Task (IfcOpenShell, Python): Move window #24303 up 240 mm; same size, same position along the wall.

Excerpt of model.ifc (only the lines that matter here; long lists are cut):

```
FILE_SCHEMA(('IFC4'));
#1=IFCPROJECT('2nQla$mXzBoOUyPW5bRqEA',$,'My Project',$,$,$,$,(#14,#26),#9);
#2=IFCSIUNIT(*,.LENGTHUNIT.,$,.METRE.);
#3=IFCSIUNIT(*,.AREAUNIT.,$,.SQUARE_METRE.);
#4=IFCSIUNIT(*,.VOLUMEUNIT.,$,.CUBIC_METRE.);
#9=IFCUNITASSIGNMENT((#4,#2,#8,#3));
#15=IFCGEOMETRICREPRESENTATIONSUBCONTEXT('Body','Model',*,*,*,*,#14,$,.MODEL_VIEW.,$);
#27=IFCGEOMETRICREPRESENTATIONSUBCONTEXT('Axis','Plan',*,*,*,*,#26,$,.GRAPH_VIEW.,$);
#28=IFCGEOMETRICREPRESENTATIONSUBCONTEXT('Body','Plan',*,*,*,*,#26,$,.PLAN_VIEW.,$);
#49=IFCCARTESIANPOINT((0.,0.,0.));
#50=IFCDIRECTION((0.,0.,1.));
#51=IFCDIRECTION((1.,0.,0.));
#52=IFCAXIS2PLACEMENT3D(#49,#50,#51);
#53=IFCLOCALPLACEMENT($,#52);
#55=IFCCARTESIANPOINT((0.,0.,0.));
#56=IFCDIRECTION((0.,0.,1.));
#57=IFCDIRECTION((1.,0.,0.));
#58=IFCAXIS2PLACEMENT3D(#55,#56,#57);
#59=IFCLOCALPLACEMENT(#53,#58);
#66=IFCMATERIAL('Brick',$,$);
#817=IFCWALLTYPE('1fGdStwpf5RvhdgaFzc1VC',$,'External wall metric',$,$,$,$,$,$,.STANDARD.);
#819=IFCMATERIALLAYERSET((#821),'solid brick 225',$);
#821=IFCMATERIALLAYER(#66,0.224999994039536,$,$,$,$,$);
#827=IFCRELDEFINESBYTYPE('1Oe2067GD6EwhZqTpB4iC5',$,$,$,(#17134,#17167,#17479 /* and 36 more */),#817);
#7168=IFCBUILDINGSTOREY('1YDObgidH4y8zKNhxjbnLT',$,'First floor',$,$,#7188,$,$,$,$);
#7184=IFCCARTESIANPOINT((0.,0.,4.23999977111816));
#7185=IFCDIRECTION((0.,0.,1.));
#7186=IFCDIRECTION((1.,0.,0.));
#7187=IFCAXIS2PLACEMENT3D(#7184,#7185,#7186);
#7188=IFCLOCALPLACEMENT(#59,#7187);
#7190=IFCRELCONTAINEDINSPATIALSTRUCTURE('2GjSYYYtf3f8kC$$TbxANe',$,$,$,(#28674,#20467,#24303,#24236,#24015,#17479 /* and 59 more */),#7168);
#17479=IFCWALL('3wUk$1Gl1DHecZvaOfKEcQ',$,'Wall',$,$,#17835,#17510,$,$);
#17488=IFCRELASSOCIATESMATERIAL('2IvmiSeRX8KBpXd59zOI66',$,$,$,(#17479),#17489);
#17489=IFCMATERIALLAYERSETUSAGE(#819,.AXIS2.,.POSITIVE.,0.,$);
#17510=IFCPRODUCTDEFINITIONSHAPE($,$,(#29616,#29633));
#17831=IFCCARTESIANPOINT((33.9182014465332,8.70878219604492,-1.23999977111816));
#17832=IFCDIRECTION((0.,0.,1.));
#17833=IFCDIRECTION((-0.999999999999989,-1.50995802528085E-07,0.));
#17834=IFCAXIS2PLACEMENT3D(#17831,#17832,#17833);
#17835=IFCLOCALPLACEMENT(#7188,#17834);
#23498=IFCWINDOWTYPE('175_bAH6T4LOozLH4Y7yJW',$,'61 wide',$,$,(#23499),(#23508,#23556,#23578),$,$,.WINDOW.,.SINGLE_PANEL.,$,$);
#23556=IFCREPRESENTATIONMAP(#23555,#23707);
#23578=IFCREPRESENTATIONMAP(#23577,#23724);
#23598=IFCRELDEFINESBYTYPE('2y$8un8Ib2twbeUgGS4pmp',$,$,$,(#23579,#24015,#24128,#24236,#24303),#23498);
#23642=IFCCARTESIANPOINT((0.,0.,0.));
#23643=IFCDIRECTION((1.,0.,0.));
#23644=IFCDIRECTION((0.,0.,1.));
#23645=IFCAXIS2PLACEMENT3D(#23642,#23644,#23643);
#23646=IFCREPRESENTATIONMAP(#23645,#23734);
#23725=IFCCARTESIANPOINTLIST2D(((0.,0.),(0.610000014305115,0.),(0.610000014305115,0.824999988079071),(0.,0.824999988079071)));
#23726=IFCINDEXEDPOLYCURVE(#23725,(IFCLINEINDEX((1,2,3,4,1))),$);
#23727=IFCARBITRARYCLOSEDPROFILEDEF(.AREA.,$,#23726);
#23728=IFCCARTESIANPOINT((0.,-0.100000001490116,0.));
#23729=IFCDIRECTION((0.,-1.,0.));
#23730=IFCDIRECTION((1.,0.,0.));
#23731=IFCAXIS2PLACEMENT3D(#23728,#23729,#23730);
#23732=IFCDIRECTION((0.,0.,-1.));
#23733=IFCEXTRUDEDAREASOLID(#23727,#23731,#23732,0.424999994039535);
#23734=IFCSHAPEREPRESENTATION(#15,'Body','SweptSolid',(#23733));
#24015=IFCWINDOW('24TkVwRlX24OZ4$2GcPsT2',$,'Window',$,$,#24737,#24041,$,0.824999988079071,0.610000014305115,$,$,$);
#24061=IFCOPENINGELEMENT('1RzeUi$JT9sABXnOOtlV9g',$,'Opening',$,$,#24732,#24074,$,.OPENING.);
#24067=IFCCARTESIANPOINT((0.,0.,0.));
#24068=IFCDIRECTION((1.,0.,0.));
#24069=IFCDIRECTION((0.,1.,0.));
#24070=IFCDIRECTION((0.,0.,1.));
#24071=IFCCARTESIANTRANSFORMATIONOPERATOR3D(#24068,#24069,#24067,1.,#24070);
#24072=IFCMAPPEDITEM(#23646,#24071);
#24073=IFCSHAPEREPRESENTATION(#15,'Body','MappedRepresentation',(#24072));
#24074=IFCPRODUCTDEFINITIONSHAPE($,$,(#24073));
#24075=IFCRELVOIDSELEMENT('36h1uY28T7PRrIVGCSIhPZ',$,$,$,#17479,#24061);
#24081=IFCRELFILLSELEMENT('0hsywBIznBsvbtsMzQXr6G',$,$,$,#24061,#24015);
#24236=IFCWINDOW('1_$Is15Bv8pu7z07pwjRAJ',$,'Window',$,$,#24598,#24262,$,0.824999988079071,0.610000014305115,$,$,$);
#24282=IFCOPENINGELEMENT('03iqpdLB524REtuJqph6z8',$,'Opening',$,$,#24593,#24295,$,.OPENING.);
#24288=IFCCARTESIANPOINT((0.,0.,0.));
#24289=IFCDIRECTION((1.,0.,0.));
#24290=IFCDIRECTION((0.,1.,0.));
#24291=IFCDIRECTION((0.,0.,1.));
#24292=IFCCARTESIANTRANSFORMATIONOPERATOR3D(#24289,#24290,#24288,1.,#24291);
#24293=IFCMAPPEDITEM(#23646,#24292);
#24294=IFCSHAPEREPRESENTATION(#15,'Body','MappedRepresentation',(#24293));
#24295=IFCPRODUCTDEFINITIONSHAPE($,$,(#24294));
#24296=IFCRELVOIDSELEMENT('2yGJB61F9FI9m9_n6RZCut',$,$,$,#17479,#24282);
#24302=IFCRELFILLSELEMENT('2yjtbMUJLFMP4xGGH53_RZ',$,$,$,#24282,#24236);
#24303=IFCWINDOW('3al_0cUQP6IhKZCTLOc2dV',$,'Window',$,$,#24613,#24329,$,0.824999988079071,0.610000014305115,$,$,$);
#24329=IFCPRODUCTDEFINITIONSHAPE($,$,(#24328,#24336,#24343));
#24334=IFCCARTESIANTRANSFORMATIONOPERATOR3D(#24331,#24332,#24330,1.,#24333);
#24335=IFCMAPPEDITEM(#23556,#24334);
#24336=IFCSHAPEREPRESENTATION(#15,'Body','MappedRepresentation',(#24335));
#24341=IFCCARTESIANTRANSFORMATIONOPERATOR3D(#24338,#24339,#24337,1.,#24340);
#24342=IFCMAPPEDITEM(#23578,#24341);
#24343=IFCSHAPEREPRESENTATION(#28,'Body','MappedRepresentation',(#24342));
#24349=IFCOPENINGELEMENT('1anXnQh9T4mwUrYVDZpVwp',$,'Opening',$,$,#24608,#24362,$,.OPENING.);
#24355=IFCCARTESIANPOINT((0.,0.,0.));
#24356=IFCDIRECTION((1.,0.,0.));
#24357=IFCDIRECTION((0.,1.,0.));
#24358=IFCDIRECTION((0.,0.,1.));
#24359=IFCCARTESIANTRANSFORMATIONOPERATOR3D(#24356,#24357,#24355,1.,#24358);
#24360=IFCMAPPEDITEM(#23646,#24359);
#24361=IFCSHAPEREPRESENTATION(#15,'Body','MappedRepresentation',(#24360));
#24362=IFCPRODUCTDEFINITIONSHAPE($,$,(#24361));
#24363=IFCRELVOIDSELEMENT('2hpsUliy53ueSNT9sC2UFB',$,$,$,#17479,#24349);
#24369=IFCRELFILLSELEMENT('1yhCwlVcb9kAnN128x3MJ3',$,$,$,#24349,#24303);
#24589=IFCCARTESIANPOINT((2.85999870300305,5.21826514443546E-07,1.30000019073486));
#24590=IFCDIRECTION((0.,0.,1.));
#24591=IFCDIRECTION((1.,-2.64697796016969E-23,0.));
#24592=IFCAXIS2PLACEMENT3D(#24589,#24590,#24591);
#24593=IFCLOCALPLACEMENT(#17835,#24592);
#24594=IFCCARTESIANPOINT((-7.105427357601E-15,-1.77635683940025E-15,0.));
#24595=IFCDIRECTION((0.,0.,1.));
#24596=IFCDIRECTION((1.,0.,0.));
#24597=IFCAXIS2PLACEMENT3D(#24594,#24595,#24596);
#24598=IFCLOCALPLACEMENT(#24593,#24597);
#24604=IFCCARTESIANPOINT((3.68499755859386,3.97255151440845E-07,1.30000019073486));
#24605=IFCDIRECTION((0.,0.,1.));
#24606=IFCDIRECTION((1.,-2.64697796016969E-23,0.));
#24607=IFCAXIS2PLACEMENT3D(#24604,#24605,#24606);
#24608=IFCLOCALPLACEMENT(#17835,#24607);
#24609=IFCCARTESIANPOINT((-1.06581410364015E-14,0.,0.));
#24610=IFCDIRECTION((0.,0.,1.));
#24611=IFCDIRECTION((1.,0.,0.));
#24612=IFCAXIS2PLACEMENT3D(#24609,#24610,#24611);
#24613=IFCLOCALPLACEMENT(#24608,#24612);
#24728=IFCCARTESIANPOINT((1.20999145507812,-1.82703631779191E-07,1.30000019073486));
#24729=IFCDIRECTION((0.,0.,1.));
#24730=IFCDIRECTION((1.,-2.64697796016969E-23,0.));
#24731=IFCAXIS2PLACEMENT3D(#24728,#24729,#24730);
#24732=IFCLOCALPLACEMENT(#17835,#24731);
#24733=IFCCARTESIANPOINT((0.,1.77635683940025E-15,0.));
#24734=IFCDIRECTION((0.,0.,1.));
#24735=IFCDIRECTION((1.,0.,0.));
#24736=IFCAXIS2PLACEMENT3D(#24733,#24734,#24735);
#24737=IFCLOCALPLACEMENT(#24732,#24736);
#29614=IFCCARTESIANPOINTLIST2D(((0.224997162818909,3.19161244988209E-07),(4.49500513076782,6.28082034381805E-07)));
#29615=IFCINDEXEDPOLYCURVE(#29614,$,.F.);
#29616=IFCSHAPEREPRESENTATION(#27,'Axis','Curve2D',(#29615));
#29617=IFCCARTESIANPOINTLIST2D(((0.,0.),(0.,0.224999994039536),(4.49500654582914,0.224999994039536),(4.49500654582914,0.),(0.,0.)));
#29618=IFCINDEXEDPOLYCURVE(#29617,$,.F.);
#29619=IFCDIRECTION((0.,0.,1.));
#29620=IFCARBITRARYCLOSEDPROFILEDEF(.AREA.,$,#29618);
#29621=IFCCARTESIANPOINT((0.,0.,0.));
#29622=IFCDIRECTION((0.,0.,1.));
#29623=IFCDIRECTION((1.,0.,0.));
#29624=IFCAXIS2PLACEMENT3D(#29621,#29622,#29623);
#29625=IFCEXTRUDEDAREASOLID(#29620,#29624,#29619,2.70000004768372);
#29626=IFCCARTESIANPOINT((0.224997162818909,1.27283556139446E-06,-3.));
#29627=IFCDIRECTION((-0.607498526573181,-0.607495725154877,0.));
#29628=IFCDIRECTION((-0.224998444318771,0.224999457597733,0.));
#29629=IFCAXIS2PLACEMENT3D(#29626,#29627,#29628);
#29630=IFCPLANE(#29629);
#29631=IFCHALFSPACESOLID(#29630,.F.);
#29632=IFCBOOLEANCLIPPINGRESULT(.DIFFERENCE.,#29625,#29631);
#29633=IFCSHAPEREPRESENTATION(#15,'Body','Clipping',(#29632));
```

```python
import numpy as np
import ifcopenshell
import ifcopenshell.api.geometry
import ifcopenshell.util.placement
import ifcopenshell.util.unit

model = ifcopenshell.open("model.ifc")
unit_scale = ifcopenshell.util.unit.calculate_unit_scale(model)

window = model.by_guid("3al_0cUQP6IhKZCTLOc2dV")
opening = window.FillsVoids[0].RelatingOpeningElement
dz = 0.24

shift = np.array([0.0, 0.0, dz])
# The window is placed relative to its opening, so it follows when the opening moves.
matrix = ifcopenshell.util.placement.get_local_placement(opening.ObjectPlacement)
matrix[:3, 3] += shift
ifcopenshell.api.geometry.edit_object_placement(
    model, product=opening, matrix=matrix, is_si=False, should_transform_children=True
)

print(f"moved by {dz * unit_scale:+.3f} m")

model.write("model_rev.ifc")
```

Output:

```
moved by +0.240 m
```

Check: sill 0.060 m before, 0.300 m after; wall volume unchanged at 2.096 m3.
